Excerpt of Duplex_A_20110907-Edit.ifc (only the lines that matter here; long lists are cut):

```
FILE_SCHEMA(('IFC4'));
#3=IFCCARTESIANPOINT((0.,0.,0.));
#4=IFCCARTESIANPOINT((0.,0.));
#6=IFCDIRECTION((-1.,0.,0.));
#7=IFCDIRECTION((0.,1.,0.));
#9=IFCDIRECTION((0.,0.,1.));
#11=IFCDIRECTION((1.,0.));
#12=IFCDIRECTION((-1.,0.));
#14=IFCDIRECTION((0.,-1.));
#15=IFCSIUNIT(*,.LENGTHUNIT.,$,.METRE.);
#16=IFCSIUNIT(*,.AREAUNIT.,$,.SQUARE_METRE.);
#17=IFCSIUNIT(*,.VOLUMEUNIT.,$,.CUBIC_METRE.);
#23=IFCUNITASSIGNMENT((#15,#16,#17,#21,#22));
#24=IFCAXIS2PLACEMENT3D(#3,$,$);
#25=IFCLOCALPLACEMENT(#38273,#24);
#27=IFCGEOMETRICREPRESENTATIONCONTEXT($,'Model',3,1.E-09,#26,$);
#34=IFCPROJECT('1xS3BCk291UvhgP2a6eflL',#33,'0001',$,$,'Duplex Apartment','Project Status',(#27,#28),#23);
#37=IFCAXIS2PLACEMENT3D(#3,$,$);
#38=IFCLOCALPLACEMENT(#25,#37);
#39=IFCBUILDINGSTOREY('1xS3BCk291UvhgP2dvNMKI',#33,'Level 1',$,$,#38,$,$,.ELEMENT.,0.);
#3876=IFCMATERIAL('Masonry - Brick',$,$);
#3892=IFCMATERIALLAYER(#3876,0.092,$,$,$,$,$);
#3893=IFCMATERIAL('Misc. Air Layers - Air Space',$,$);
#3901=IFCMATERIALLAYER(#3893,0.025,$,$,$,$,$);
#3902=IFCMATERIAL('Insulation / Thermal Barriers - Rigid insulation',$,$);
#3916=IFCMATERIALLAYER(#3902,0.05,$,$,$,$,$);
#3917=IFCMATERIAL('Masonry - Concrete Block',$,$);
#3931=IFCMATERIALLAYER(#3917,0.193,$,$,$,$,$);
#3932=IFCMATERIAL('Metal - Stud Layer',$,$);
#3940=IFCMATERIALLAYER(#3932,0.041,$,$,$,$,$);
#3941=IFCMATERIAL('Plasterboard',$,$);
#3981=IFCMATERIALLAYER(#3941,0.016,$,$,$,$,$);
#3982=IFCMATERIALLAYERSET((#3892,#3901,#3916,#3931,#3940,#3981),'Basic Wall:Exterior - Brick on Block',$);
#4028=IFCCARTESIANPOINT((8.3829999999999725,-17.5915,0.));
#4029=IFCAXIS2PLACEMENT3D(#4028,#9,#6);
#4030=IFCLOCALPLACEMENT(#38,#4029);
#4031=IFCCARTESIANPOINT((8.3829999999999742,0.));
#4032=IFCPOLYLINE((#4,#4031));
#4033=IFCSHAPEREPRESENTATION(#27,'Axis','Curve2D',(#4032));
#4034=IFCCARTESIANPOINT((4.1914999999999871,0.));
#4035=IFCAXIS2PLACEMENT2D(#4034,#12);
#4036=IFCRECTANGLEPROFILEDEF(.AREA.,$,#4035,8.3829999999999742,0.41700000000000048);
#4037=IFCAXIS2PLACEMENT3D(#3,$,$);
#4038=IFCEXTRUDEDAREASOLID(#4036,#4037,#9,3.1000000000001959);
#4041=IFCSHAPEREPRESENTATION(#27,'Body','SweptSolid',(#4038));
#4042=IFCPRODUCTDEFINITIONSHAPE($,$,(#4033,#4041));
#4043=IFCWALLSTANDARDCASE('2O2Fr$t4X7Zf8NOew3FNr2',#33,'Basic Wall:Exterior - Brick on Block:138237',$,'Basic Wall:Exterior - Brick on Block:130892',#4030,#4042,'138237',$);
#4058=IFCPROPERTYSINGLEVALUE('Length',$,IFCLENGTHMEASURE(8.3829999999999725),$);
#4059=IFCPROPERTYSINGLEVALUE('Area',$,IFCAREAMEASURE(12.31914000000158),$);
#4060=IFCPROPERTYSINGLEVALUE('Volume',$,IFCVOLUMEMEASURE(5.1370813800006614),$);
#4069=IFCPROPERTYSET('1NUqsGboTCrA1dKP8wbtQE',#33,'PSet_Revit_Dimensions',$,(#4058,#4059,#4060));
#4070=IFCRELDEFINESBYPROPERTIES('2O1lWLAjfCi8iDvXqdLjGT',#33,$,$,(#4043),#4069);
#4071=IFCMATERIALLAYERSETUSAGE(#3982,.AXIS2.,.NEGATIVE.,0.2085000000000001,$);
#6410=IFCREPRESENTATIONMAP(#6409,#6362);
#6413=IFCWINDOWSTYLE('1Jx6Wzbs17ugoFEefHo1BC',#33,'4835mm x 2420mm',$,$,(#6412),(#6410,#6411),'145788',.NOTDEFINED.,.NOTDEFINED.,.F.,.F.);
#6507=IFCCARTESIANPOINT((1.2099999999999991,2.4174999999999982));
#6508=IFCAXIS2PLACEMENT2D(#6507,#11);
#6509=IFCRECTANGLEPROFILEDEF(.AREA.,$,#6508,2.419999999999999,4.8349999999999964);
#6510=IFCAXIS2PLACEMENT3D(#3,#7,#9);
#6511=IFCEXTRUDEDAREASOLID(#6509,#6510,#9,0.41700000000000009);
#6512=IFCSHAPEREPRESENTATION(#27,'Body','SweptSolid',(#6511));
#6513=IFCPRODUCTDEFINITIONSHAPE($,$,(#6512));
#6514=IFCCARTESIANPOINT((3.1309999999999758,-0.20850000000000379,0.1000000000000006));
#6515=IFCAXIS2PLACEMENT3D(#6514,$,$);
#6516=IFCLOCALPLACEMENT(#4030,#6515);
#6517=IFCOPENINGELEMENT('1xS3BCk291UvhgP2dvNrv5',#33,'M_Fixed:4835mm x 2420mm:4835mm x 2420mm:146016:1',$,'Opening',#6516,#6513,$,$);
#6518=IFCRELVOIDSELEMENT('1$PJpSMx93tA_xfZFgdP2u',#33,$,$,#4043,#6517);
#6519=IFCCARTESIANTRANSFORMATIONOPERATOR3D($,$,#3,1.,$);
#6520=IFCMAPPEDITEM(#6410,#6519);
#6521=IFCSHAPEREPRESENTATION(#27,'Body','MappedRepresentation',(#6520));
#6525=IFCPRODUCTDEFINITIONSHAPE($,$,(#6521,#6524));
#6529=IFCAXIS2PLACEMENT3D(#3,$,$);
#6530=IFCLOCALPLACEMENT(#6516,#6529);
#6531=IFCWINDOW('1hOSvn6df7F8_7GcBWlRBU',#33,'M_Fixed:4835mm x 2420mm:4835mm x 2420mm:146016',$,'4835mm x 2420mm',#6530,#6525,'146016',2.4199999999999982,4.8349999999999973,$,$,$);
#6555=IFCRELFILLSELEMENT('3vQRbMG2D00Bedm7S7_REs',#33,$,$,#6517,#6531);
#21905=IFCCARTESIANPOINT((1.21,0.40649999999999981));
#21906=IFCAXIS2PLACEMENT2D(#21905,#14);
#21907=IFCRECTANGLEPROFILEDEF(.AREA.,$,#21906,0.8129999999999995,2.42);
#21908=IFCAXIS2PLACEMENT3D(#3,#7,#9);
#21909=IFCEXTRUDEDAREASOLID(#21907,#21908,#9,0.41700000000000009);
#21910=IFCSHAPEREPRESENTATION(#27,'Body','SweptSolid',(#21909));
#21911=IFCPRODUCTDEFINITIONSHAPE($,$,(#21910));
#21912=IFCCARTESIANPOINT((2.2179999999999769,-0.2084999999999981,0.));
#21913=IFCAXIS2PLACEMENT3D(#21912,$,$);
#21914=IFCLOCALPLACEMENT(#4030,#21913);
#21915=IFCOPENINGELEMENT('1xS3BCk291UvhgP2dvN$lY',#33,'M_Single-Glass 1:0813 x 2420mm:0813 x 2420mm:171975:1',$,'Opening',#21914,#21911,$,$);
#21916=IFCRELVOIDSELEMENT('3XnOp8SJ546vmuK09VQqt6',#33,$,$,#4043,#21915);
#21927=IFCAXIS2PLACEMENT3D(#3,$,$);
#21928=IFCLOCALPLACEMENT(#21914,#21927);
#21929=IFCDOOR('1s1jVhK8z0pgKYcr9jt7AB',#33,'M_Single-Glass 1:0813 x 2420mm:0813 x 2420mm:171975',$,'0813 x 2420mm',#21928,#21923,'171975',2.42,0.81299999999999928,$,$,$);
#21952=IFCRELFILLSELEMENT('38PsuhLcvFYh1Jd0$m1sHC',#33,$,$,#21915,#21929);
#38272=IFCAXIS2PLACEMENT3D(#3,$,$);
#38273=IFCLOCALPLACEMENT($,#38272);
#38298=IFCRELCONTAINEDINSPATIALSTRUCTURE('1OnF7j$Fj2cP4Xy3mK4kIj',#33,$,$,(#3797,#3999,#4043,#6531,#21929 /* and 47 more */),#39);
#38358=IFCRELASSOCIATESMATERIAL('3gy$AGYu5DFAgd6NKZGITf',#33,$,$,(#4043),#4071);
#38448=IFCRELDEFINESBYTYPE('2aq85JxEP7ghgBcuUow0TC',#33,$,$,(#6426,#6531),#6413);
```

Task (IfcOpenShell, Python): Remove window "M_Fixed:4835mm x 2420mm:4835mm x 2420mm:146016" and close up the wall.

```python
import ifcopenshell
import ifcopenshell.api.feature
import ifcopenshell.api.pset
import ifcopenshell.api.root
import ifcopenshell.geom
import ifcopenshell.util.element
import ifcopenshell.util.shape
import ifcopenshell.util.unit

model = ifcopenshell.open("Duplex_A_20110907-Edit.ifc")
area_scale = ifcopenshell.util.unit.calculate_unit_scale(model, "AREAUNIT")
volume_scale = ifcopenshell.util.unit.calculate_unit_scale(model, "VOLUMEUNIT")
settings = ifcopenshell.geom.settings()


def volume(element):
    """Net volume in cubic metres, openings subtracted."""
    shape = ifcopenshell.geom.create_shape(settings, element)
    return ifcopenshell.util.shape.get_volume(shape.geometry)


window = model.by_guid("1hOSvn6df7F8_7GcBWlRBU")
opening = window.FillsVoids[0].RelatingOpeningElement
wall = opening.VoidsElements[0].RelatingBuildingElement
before = volume(wall)

ifcopenshell.api.root.remove_product(model, product=window)
ifcopenshell.api.feature.remove_feature(model, feature=opening)

after = volume(wall)
thickness = 0.417  # wall thickness in metres

# Update the wall's stored quantities.
pset = model.by_id(ifcopenshell.util.element.get_pset(wall, "PSet_Revit_Dimensions", should_inherit=False)["id"])
ifcopenshell.api.pset.edit_pset(model, pset=pset, properties={
    "Area": model.create_entity("IfcAreaMeasure", after / thickness / area_scale),
    "Volume": model.create_entity("IfcVolumeMeasure", after / volume_scale),
})

print(f"wall volume {before:.3f} -> {after:.3f} m3")

model.write("Duplex_A_20110907-Edit_v2.ifc")
```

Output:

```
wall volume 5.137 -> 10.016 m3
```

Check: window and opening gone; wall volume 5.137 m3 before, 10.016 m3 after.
